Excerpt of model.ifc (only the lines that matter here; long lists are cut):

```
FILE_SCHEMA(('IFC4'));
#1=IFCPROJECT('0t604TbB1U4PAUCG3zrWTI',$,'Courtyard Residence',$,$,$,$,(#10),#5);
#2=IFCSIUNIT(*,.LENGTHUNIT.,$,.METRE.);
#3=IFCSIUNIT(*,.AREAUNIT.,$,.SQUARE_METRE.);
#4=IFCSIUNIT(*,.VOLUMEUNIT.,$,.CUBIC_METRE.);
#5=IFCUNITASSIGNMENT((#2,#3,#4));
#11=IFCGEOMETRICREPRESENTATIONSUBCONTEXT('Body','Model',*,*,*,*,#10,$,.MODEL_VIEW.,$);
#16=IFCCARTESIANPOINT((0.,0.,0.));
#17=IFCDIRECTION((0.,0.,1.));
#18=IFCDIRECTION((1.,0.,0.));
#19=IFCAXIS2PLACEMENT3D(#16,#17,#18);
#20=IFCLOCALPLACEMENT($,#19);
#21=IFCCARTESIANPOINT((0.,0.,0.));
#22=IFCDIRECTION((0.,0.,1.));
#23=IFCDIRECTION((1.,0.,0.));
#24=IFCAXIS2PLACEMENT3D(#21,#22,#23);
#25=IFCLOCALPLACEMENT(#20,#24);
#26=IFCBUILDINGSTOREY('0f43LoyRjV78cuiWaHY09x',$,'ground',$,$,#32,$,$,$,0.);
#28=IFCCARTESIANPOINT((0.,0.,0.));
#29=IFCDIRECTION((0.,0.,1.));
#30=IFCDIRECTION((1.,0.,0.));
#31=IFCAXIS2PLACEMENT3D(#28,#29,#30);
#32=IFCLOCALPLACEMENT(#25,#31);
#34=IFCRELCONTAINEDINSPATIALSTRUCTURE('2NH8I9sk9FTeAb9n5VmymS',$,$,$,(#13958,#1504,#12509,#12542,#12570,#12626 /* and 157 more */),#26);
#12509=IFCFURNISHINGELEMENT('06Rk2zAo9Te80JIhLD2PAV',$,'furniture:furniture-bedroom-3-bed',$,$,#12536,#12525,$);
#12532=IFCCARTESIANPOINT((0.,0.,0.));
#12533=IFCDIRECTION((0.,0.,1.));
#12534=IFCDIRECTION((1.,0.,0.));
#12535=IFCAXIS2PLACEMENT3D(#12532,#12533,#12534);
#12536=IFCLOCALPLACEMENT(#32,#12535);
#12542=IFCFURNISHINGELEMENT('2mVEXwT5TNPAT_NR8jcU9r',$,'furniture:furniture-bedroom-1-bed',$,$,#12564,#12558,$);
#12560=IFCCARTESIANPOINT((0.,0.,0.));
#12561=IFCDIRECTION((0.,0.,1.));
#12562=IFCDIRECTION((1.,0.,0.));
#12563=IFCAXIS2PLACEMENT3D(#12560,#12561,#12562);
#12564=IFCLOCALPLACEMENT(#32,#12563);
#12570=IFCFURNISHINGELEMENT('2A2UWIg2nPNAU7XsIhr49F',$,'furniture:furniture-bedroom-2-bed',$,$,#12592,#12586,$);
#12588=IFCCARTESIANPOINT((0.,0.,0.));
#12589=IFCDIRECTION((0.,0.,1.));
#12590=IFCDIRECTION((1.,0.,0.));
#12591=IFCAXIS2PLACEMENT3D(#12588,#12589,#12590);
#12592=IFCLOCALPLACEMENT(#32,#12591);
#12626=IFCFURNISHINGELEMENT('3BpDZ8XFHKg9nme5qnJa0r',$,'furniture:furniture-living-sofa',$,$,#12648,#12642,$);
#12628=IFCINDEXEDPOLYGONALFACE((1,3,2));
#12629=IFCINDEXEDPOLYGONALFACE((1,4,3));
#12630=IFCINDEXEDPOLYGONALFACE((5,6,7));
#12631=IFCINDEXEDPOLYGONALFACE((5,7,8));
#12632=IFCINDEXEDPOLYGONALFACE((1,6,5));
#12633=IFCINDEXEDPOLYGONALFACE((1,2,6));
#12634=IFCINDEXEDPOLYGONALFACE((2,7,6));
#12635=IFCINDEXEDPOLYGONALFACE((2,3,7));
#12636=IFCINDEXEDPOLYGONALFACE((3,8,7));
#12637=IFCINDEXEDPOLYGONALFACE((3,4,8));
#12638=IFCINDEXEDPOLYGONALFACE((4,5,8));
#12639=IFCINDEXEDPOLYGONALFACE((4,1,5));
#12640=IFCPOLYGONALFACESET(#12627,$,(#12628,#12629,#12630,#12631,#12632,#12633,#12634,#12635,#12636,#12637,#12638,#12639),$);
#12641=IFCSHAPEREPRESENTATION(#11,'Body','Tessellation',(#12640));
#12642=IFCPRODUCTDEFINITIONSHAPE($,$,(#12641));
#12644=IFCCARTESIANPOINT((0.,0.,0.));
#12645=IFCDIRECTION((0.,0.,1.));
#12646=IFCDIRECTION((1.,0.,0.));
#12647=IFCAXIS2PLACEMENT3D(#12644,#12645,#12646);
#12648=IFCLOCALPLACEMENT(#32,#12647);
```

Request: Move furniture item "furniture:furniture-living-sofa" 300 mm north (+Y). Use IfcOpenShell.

```python
import ifcopenshell
import ifcopenshell.api.geometry
import ifcopenshell.util.placement

model = ifcopenshell.open("model.ifc")

item = model.by_guid("3BpDZ8XFHKg9nme5qnJa0r")
matrix = ifcopenshell.util.placement.get_local_placement(item.ObjectPlacement)
matrix[1, 3] += 0.3
ifcopenshell.api.geometry.edit_object_placement(model, product=item, matrix=matrix, is_si=False)

print(ifcopenshell.util.placement.get_local_placement(item.ObjectPlacement).round(3) + 0.0)

model.write("model_v2.ifc")
```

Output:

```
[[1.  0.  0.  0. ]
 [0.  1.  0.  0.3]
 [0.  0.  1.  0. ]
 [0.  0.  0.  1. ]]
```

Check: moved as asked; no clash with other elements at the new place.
